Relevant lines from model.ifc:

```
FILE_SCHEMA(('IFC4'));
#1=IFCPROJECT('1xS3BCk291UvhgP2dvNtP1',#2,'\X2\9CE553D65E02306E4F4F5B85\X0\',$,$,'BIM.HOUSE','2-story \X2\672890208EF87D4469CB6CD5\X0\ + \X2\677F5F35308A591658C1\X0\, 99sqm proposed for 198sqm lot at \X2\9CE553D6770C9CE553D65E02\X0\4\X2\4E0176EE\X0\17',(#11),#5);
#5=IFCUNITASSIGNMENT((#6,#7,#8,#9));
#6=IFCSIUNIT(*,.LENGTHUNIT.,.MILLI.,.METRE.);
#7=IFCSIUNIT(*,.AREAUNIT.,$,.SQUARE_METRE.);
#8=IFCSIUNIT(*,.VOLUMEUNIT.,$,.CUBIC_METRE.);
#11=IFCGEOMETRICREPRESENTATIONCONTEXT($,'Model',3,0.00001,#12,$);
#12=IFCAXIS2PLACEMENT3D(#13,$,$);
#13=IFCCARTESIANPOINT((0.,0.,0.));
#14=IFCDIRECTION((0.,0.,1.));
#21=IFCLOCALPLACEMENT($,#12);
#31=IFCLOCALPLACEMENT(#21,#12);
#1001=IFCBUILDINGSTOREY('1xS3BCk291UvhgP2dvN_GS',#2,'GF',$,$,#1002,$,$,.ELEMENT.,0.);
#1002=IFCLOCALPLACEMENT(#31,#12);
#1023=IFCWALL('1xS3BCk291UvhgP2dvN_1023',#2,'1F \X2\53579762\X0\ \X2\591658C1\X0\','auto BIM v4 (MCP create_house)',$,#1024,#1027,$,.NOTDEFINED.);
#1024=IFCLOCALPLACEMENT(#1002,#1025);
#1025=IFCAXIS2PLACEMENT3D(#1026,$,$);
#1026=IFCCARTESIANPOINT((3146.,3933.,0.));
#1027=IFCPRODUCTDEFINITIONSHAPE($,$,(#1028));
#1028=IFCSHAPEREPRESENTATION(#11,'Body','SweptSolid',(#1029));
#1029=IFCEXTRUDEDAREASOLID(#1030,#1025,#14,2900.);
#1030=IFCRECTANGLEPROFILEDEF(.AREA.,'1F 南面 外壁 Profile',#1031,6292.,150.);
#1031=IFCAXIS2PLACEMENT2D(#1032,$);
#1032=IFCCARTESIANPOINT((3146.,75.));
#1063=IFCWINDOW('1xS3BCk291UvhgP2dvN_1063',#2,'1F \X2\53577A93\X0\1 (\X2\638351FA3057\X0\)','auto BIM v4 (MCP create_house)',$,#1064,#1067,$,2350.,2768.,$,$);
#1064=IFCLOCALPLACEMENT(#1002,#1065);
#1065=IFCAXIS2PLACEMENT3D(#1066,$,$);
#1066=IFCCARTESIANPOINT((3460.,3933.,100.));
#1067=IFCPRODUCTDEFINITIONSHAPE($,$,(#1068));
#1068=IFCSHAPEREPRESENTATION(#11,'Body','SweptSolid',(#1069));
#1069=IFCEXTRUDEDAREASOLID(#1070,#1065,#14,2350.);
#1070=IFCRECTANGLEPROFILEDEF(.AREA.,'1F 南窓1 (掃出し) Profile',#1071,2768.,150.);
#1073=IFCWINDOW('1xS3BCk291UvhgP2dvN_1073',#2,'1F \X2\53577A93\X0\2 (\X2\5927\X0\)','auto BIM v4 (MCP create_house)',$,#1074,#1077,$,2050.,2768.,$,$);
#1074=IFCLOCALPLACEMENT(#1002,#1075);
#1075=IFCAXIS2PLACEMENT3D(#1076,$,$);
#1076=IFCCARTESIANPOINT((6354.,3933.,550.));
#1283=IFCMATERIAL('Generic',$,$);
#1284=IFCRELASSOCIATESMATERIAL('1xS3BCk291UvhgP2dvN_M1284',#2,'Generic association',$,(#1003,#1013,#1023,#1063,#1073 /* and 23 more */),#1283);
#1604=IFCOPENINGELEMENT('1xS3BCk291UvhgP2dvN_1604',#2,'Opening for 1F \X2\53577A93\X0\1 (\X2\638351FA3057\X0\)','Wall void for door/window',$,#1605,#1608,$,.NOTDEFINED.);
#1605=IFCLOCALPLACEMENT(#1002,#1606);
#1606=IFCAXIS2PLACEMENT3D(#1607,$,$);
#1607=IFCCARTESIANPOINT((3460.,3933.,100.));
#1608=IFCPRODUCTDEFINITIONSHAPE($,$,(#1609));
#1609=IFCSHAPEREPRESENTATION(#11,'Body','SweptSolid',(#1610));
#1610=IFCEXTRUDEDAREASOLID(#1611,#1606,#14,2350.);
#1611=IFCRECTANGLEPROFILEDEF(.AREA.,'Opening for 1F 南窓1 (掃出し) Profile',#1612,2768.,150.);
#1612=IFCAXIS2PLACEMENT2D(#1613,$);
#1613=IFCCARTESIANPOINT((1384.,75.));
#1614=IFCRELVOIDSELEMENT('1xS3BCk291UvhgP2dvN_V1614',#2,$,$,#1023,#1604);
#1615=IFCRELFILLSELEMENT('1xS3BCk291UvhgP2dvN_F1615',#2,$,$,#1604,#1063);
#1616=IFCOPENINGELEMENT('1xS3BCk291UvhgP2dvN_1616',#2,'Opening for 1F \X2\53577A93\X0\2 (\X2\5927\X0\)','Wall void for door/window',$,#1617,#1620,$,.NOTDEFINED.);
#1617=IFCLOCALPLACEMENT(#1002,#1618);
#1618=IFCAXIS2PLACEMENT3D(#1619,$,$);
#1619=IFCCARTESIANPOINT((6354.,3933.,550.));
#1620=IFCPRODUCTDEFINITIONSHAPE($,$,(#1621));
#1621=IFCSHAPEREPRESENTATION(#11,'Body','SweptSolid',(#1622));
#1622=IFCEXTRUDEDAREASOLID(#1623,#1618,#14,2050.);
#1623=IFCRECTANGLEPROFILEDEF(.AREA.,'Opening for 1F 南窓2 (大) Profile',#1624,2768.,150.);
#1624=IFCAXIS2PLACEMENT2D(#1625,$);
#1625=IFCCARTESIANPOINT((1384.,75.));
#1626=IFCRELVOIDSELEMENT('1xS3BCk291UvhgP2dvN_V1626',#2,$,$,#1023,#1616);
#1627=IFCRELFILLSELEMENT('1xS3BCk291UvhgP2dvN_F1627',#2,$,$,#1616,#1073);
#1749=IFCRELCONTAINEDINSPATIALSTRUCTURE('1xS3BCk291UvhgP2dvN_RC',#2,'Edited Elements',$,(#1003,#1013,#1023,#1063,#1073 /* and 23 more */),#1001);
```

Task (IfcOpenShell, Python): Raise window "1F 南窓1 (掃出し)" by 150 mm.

```python
import numpy as np
import ifcopenshell
import ifcopenshell.api.geometry
import ifcopenshell.util.placement
import ifcopenshell.util.unit

model = ifcopenshell.open("model.ifc")
unit_scale = ifcopenshell.util.unit.calculate_unit_scale(model)

window = model.by_id(1063)
opening = window.FillsVoids[0].RelatingOpeningElement
dz = 0.15 / unit_scale

shift = np.array([0.0, 0.0, dz])
# The window is not placed relative to its opening, so move both.
for product in (opening, window):
    matrix = ifcopenshell.util.placement.get_local_placement(product.ObjectPlacement)
    matrix[:3, 3] += shift
    ifcopenshell.api.geometry.edit_object_placement(model, product=product, matrix=matrix, is_si=False)

print(f"moved by {dz * unit_scale:+.3f} m")

model.write("model_v2.ifc")
```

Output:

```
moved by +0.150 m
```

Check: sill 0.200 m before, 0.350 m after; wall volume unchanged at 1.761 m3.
